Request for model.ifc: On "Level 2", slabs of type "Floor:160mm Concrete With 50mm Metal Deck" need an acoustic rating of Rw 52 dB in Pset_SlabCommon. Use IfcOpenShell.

First a look at what the model holds.

```python
import ifcopenshell
import ifcopenshell.util.element

model = ifcopenshell.open("model.ifc")
print(model.schema)
storey = next(s for s in model.by_type("IfcBuildingStorey") if s.Name == "Level 2")
slabs = [e for e in ifcopenshell.util.element.get_decomposition(storey) if e.is_a("IfcSlab")]
seen = {}
for e in slabs:
    element_type = ifcopenshell.util.element.get_type(e)
    key = (element_type.Name if element_type != e and element_type else None, ifcopenshell.util.element.get_pset(e, "Pset_SlabCommon", "AcousticRating"))
    seen[key] = seen.get(key, 0) + 1
for (name, value), count in sorted(seen.items(), key=str):
    print(count, "x", name, "|", value)
```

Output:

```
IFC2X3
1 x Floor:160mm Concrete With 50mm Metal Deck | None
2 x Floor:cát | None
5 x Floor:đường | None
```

```python
import ifcopenshell
import ifcopenshell.api.pset
import ifcopenshell.util.element

model = ifcopenshell.open("model.ifc")

storey = next(s for s in model.by_type("IfcBuildingStorey") if s.Name == "Level 2")
slabs = [e for e in ifcopenshell.util.element.get_decomposition(storey) if e.is_a("IfcSlab")]

count = 0
for e in slabs:
    element_type = ifcopenshell.util.element.get_type(e)
    if element_type in (None, e) or element_type.Name != "Floor:160mm Concrete With 50mm Metal Deck":
        continue
    # add_pset returns the element's existing set when there is one.
    pset = ifcopenshell.api.pset.add_pset(model, product=e, name="Pset_SlabCommon")
    ifcopenshell.api.pset.edit_pset(model, pset=pset, properties={"AcousticRating": "Rw 52 dB"})
    count += 1

print(count, "slabs updated")

model.write("model_updated.ifc")
```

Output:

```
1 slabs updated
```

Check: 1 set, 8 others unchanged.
